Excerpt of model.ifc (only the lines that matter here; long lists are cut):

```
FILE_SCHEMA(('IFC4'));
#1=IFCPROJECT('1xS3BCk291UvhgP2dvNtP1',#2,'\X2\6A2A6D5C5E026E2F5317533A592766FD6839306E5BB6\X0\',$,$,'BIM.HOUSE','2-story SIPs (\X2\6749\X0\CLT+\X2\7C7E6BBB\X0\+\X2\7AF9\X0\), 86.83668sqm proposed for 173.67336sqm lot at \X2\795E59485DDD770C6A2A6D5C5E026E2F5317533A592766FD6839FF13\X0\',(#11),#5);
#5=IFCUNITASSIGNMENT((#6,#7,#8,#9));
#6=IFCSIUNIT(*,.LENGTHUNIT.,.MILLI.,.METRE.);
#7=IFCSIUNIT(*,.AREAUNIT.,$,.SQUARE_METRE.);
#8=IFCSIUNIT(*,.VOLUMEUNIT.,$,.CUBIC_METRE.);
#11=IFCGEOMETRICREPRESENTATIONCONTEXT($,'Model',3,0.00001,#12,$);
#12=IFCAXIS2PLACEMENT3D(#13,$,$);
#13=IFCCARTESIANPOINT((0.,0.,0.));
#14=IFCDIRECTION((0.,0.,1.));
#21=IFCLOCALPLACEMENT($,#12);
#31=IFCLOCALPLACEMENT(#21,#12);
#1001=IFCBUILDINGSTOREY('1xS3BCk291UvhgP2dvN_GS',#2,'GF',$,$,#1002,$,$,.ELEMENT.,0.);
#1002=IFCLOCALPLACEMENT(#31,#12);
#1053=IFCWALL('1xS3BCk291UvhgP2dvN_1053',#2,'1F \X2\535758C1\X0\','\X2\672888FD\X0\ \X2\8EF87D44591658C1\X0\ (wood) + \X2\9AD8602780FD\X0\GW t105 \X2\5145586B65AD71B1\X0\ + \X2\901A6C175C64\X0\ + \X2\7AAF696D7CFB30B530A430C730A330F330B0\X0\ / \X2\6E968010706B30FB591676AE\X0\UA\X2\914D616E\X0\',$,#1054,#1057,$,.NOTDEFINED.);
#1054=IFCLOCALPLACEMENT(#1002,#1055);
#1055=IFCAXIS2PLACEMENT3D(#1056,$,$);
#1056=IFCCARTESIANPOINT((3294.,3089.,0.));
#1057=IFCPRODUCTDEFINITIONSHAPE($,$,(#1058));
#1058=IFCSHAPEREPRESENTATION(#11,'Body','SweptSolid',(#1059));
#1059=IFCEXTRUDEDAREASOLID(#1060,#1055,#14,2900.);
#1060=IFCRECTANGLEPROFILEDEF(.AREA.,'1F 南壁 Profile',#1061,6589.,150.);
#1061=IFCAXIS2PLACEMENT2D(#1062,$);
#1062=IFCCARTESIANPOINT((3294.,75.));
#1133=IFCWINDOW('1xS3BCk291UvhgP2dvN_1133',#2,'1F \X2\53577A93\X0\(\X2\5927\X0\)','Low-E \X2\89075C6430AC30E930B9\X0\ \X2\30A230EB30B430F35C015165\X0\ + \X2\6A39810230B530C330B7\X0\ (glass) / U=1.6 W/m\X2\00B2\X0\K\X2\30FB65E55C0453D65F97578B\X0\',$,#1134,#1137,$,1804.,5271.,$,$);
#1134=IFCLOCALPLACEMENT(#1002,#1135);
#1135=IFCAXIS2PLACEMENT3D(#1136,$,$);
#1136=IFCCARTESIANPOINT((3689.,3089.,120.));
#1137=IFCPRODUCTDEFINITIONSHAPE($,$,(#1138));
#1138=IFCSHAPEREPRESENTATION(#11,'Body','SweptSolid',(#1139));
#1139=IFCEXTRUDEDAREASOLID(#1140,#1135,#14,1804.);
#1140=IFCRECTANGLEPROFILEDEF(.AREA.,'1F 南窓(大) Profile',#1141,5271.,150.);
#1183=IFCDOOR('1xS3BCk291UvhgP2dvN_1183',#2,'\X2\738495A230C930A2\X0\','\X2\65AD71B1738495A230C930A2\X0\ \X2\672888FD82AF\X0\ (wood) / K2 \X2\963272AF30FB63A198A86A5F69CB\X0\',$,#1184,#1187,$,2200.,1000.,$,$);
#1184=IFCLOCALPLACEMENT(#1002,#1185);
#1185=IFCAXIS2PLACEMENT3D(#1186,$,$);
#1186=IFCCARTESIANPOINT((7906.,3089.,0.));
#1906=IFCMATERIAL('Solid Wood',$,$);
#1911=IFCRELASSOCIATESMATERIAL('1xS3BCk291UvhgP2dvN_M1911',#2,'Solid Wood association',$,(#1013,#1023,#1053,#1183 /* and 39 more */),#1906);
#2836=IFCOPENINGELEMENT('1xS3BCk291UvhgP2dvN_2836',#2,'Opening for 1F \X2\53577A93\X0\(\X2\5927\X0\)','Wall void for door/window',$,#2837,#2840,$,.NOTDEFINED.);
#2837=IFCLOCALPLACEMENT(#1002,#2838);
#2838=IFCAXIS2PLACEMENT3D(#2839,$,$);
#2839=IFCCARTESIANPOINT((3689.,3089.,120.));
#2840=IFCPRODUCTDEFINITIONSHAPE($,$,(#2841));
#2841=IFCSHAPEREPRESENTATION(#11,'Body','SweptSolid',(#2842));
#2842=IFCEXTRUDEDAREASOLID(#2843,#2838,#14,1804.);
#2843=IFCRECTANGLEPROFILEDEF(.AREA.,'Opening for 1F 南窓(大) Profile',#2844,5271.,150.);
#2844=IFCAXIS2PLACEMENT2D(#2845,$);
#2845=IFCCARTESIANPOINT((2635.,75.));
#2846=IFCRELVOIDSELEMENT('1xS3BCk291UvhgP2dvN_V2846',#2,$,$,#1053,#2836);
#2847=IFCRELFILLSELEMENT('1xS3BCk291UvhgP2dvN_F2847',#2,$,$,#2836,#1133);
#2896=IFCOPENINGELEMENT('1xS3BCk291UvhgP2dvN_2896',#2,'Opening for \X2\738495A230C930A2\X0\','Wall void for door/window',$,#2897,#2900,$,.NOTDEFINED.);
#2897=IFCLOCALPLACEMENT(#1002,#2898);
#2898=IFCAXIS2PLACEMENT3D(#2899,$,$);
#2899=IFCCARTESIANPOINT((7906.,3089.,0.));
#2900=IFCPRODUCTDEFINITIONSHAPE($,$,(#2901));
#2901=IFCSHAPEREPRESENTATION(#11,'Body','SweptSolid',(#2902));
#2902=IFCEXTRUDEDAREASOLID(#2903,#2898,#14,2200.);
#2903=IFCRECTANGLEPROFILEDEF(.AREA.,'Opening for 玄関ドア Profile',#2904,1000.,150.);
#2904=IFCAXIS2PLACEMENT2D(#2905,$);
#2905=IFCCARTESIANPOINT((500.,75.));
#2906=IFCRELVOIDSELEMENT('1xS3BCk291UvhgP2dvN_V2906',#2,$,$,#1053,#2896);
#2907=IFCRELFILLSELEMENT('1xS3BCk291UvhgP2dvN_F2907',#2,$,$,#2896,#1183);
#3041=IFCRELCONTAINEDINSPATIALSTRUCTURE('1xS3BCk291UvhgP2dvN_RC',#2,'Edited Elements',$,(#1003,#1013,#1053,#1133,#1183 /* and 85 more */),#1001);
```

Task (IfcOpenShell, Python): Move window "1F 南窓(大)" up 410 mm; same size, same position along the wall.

```python
import numpy as np
import ifcopenshell
import ifcopenshell.api.geometry
import ifcopenshell.util.placement
import ifcopenshell.util.unit

model = ifcopenshell.open("model.ifc")
unit_scale = ifcopenshell.util.unit.calculate_unit_scale(model)

window = model.by_guid("1xS3BCk291UvhgP2dvN_1133")
opening = window.FillsVoids[0].RelatingOpeningElement
dz = 0.41 / unit_scale

shift = np.array([0.0, 0.0, dz])
# The window is not placed relative to its opening, so move both.
for product in (opening, window):
    matrix = ifcopenshell.util.placement.get_local_placement(product.ObjectPlacement)
    matrix[:3, 3] += shift
    ifcopenshell.api.geometry.edit_object_placement(model, product=product, matrix=matrix, is_si=False)

print(f"moved by {dz * unit_scale:+.3f} m")

model.write("model_v2.ifc")
```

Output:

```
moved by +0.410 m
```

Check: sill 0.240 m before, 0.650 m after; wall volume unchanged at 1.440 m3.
